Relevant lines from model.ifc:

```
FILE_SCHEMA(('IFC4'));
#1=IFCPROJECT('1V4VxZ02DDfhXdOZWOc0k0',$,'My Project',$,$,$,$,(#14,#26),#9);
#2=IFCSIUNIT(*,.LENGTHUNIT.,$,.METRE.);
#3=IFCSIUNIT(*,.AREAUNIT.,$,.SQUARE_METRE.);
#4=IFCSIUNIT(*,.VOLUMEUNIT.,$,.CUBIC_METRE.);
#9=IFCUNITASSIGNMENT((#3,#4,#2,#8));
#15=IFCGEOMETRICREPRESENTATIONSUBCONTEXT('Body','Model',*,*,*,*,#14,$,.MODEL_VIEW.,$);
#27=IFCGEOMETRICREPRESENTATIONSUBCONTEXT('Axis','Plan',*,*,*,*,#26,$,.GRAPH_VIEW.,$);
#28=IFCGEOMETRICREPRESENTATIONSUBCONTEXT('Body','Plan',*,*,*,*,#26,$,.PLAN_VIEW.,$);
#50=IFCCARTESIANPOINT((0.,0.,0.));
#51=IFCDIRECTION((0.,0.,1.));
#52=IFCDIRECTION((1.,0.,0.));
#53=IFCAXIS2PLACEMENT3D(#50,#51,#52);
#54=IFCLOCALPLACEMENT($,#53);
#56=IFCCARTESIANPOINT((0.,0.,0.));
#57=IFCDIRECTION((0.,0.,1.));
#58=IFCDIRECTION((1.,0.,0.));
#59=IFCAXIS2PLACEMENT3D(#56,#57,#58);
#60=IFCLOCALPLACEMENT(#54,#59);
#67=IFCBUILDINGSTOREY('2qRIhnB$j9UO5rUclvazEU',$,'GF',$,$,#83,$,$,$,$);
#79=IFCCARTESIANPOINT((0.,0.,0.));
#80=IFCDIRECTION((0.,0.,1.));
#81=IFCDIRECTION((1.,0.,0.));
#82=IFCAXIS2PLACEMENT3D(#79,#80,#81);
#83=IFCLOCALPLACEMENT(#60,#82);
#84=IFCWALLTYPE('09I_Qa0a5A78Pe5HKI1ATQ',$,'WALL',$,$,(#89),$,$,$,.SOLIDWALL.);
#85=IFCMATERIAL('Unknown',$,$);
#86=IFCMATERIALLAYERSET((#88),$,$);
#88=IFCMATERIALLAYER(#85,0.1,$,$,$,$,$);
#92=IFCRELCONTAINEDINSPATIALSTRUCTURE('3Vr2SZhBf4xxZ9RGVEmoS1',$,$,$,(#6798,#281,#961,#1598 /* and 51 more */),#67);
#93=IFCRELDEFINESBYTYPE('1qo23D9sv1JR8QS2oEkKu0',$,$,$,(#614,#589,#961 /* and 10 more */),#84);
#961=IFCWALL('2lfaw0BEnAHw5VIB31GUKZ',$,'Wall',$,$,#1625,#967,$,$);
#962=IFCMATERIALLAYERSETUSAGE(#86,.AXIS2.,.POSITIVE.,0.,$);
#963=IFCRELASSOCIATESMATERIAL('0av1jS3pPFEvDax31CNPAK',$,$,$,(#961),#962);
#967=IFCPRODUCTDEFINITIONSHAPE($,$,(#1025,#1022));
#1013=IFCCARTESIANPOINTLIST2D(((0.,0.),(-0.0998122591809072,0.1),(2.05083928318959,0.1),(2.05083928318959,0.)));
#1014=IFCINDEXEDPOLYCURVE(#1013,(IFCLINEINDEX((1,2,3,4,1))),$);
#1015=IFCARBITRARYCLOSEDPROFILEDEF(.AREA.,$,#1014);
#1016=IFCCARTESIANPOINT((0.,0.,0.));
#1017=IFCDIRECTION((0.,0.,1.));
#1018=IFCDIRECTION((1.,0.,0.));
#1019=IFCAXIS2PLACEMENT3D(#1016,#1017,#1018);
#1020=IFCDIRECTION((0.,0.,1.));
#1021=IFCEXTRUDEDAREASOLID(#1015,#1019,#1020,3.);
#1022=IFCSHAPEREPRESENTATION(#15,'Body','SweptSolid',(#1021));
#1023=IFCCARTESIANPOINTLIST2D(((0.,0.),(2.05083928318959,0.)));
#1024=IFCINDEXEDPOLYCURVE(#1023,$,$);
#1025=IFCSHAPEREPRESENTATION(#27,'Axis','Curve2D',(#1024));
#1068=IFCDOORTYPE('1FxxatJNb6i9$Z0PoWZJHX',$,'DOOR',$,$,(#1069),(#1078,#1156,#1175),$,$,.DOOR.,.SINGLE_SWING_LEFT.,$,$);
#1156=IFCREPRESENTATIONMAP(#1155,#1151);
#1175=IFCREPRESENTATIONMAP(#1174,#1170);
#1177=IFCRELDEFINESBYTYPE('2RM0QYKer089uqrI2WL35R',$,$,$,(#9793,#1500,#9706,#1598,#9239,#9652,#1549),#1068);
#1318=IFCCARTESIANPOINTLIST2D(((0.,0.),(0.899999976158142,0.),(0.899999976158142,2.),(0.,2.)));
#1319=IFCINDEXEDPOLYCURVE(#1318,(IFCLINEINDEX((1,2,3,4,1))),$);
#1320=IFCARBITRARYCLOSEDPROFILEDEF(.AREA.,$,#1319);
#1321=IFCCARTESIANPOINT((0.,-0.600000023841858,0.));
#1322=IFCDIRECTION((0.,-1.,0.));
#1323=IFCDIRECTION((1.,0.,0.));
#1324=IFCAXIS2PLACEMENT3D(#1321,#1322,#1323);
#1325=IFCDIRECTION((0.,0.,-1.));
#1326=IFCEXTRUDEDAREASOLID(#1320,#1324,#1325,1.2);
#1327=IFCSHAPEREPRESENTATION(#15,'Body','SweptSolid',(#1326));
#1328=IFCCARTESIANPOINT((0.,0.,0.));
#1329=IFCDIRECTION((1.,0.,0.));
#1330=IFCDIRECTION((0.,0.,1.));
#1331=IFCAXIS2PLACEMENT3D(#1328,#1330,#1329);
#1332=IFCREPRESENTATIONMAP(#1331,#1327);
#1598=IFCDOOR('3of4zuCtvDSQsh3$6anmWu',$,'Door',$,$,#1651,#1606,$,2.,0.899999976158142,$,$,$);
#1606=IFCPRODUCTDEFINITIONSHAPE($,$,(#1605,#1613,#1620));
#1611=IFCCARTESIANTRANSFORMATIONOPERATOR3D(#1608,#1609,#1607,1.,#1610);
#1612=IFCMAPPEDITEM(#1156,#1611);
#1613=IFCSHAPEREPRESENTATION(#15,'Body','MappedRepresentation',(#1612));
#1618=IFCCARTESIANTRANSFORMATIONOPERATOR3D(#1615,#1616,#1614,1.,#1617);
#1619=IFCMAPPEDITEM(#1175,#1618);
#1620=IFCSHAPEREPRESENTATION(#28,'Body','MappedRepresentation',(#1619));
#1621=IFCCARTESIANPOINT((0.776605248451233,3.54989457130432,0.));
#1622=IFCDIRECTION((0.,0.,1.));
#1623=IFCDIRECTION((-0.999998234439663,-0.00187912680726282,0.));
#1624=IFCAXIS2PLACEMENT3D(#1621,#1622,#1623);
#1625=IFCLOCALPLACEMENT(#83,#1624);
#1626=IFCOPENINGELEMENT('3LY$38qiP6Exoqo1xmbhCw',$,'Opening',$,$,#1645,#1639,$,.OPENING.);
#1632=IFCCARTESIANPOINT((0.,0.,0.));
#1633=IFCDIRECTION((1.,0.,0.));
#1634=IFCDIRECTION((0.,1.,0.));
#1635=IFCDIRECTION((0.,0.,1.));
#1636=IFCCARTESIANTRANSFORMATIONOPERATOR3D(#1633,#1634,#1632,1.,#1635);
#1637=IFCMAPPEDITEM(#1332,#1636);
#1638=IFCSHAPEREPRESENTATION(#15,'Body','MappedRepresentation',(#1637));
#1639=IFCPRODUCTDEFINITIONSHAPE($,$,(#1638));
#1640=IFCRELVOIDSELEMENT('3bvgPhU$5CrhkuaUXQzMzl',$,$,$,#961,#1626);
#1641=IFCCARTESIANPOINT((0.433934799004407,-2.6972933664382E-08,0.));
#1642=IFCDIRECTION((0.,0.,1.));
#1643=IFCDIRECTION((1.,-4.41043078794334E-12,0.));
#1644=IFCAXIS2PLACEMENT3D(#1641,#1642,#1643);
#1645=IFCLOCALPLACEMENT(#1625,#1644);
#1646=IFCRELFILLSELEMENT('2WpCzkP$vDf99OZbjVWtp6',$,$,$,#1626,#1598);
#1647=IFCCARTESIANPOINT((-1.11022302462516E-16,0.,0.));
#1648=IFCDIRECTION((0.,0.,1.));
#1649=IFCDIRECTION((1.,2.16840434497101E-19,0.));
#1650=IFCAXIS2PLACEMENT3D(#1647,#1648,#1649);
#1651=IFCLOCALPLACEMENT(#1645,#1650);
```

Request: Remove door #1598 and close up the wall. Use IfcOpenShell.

```python
import ifcopenshell
import ifcopenshell.api.feature
import ifcopenshell.api.root
import ifcopenshell.geom
import ifcopenshell.util.shape

model = ifcopenshell.open("model.ifc")
settings = ifcopenshell.geom.settings()


def volume(element):
    """Net volume in cubic metres, openings subtracted."""
    shape = ifcopenshell.geom.create_shape(settings, element)
    return ifcopenshell.util.shape.get_volume(shape.geometry)


door = model.by_guid("3of4zuCtvDSQsh3$6anmWu")
opening = door.FillsVoids[0].RelatingOpeningElement
wall = opening.VoidsElements[0].RelatingBuildingElement
before = volume(wall)

ifcopenshell.api.root.remove_product(model, product=door)
ifcopenshell.api.feature.remove_feature(model, feature=opening)

after = volume(wall)

print(f"wall volume {before:.3f} -> {after:.3f} m3")

model.write("model-out.ifc")
```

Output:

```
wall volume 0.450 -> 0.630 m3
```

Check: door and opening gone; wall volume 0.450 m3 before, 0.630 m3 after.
